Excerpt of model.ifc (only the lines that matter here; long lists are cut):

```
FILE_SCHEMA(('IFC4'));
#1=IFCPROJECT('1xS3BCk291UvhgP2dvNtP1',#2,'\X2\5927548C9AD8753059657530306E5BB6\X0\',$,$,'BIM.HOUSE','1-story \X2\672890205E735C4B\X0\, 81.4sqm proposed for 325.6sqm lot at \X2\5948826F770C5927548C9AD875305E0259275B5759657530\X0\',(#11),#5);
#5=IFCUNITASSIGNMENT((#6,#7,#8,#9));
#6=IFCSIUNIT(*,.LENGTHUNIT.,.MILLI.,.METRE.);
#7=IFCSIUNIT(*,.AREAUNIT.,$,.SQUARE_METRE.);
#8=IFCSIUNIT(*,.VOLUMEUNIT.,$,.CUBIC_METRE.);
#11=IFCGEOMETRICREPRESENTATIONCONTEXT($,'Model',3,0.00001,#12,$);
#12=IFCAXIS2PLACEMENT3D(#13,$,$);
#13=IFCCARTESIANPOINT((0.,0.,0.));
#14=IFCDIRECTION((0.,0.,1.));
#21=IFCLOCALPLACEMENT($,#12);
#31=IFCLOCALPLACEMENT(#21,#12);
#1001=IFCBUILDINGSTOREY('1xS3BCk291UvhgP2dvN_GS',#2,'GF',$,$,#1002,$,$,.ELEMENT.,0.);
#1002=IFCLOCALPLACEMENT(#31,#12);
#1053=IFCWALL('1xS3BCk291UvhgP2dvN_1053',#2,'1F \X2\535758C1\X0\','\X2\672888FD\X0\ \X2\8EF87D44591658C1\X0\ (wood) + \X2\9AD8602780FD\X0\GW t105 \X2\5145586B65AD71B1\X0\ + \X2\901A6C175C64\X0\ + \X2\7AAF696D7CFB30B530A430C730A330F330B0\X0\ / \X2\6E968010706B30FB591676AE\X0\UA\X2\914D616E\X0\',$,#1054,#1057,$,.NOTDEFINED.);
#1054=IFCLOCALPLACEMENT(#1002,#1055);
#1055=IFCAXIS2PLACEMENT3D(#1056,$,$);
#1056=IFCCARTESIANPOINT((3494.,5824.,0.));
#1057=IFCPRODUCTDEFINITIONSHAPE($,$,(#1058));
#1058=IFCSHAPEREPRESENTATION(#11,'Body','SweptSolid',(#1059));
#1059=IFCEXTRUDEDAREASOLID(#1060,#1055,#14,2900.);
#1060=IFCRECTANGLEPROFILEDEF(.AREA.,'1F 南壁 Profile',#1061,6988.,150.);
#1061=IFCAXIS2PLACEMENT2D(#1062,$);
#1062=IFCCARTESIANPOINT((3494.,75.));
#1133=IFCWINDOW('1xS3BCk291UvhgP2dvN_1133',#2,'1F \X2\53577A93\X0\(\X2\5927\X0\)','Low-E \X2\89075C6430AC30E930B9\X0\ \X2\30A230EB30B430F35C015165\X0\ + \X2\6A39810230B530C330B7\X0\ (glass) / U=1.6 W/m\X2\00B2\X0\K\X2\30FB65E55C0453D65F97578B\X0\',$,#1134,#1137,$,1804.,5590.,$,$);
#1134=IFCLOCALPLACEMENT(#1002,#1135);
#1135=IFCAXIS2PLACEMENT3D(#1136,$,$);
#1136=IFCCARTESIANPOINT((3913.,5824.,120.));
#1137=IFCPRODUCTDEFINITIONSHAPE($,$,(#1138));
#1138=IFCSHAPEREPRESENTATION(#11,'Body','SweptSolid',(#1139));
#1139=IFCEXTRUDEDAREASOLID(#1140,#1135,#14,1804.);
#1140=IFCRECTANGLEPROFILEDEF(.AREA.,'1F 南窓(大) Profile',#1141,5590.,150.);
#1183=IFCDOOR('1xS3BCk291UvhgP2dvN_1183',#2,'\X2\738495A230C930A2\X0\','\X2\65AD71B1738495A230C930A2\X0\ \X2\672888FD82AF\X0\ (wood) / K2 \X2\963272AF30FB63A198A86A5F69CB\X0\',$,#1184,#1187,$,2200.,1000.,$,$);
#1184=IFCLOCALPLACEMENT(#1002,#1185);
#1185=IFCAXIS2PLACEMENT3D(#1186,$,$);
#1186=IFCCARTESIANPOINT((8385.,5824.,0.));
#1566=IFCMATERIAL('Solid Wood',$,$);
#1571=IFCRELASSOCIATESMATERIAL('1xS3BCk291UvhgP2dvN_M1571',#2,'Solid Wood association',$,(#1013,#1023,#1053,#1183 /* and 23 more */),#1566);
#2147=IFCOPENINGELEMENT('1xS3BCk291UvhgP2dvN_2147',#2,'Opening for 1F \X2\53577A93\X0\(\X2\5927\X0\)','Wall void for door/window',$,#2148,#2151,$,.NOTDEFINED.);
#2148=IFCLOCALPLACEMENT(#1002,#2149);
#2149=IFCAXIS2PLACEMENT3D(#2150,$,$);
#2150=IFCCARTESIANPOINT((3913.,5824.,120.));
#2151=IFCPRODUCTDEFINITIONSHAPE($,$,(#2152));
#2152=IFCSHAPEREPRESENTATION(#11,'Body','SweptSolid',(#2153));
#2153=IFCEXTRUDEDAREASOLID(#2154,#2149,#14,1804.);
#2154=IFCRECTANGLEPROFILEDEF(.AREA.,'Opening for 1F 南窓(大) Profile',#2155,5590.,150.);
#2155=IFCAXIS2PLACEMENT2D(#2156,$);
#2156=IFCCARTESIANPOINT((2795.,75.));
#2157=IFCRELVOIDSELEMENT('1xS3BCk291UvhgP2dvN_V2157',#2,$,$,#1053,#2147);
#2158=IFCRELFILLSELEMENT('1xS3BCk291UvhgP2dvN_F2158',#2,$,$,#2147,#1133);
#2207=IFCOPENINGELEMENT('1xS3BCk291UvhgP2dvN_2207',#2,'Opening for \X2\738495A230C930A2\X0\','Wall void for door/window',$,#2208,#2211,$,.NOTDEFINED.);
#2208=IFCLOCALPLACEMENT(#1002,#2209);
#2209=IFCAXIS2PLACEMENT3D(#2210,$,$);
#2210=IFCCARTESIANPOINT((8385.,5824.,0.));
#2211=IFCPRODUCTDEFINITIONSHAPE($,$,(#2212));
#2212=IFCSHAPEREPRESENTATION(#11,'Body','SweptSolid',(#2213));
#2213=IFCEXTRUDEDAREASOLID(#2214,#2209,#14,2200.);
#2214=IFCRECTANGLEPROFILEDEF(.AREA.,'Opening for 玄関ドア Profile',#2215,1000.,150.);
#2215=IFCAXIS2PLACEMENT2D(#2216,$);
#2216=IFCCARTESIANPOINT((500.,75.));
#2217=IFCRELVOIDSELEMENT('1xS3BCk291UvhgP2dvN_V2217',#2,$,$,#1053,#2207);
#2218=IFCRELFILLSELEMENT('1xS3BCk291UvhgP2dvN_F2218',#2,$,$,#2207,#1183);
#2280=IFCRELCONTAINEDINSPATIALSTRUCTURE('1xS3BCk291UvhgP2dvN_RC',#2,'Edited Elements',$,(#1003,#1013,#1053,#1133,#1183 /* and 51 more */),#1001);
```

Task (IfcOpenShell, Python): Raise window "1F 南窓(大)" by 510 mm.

```python
import numpy as np
import ifcopenshell
import ifcopenshell.api.geometry
import ifcopenshell.util.placement
import ifcopenshell.util.unit

model = ifcopenshell.open("model.ifc")
unit_scale = ifcopenshell.util.unit.calculate_unit_scale(model)

window = model.by_id(1133)
opening = window.FillsVoids[0].RelatingOpeningElement
dz = 510.0

shift = np.array([0.0, 0.0, dz])
# The window is not placed relative to its opening, so move both.
for product in (opening, window):
    matrix = ifcopenshell.util.placement.get_local_placement(product.ObjectPlacement)
    matrix[:3, 3] += shift
    ifcopenshell.api.geometry.edit_object_placement(model, product=product, matrix=matrix, is_si=False)

print(f"moved by {dz * unit_scale:+.3f} m")

model.write("model_updated.ifc")
```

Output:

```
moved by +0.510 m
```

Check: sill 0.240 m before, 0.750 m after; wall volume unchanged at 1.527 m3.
